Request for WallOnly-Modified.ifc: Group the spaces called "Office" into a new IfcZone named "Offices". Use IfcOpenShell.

First a look at what the model holds.

```python
import ifcopenshell

model = ifcopenshell.open("WallOnly-Modified.ifc")
print(model.schema)
seen = {}
for space in model.by_type("IfcSpace"):
    seen[space.LongName] = seen.get(space.LongName, 0) + 1
for name, count in sorted(seen.items(), key=str):
    print(count, "x", name)
print("zones:", [z.Name for z in model.by_type("IfcZone")][:20])
```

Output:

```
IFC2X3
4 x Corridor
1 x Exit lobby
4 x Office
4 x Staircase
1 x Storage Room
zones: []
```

```python
import ifcopenshell
import ifcopenshell.api.group
import ifcopenshell.api.root

model = ifcopenshell.open("WallOnly-Modified.ifc")

names = {"Office"}
spaces = [s for s in model.by_type("IfcSpace") if s.LongName in names]

zone = ifcopenshell.api.root.create_entity(model, ifc_class="IfcZone", name="Offices")
ifcopenshell.api.group.assign_group(model, products=spaces, group=zone)
print(len(spaces), "spaces in", zone.Name)

model.write("WallOnly-Modified_v2.ifc")
```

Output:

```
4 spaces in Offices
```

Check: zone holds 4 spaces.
